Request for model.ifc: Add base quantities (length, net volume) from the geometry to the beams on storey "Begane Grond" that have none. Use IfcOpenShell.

First a look at what the model holds.

```python
import ifcopenshell
import ifcopenshell.util.element
import ifcopenshell.util.unit

model = ifcopenshell.open("model.ifc")
print(model.schema)
for unit_type in ("LENGTHUNIT", "AREAUNIT", "VOLUMEUNIT"):
    print(unit_type, ifcopenshell.util.unit.calculate_unit_scale(model, unit_type))
storey = next(s for s in model.by_type("IfcBuildingStorey") if s.Name == "Begane Grond")
beams = [e for e in ifcopenshell.util.element.get_decomposition(storey) if e.is_a("IfcBeam")]
for e in sorted(beams, key=lambda e: e.id()):
    print(e.id(), e.is_a(), e.Name, list(ifcopenshell.util.element.get_psets(e, qtos_only=True)), sep=" | ")
```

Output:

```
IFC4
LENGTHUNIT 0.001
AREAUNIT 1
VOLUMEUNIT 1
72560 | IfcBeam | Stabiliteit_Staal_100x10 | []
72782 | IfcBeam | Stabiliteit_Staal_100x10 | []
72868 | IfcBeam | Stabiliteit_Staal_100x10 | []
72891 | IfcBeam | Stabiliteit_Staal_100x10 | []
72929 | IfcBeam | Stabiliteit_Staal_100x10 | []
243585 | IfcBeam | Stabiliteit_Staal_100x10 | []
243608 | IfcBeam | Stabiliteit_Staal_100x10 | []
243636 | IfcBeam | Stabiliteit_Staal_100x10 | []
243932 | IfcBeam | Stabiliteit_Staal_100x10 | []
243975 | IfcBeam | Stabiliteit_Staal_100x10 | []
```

```python
import ifcopenshell
import ifcopenshell.api.pset
import ifcopenshell.geom
import ifcopenshell.util.element
import ifcopenshell.util.shape
import ifcopenshell.util.unit

model = ifcopenshell.open("model.ifc")
unit_scale = ifcopenshell.util.unit.calculate_unit_scale(model)
volume_scale = ifcopenshell.util.unit.calculate_unit_scale(model, "VOLUMEUNIT")
settings = ifcopenshell.geom.settings()

storey = next(s for s in model.by_type("IfcBuildingStorey") if s.Name == "Begane Grond")
beams = [e for e in ifcopenshell.util.element.get_decomposition(storey) if e.is_a("IfcBeam")]

for e in sorted(beams, key=lambda e: e.id()):
    if ifcopenshell.util.element.get_psets(e, qtos_only=True, should_inherit=False):
        continue
    # Geometry comes back in metres, in the element's own axes.
    shape = ifcopenshell.geom.create_shape(settings, e)
    values = {
        "Length": ifcopenshell.util.shape.get_max_xyz(shape.geometry) / unit_scale,
        "NetVolume": ifcopenshell.util.shape.get_volume(shape.geometry) / volume_scale,
    }
    qto = ifcopenshell.api.pset.add_qto(model, product=e, name="Qto_BeamBaseQuantities")
    ifcopenshell.api.pset.edit_qto(model, qto=qto, properties=values)
    print(e.id(), {k: round(v, 3) for k, v in values.items()})

model.write("model_v2.ifc")
```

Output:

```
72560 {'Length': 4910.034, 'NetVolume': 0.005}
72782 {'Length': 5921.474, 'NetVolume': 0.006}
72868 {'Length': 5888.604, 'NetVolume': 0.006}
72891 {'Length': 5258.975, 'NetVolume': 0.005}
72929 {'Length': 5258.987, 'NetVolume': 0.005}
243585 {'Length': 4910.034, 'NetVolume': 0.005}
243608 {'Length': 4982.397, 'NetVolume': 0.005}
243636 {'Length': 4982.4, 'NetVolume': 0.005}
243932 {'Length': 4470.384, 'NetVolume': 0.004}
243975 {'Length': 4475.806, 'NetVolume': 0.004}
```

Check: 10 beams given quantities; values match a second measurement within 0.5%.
